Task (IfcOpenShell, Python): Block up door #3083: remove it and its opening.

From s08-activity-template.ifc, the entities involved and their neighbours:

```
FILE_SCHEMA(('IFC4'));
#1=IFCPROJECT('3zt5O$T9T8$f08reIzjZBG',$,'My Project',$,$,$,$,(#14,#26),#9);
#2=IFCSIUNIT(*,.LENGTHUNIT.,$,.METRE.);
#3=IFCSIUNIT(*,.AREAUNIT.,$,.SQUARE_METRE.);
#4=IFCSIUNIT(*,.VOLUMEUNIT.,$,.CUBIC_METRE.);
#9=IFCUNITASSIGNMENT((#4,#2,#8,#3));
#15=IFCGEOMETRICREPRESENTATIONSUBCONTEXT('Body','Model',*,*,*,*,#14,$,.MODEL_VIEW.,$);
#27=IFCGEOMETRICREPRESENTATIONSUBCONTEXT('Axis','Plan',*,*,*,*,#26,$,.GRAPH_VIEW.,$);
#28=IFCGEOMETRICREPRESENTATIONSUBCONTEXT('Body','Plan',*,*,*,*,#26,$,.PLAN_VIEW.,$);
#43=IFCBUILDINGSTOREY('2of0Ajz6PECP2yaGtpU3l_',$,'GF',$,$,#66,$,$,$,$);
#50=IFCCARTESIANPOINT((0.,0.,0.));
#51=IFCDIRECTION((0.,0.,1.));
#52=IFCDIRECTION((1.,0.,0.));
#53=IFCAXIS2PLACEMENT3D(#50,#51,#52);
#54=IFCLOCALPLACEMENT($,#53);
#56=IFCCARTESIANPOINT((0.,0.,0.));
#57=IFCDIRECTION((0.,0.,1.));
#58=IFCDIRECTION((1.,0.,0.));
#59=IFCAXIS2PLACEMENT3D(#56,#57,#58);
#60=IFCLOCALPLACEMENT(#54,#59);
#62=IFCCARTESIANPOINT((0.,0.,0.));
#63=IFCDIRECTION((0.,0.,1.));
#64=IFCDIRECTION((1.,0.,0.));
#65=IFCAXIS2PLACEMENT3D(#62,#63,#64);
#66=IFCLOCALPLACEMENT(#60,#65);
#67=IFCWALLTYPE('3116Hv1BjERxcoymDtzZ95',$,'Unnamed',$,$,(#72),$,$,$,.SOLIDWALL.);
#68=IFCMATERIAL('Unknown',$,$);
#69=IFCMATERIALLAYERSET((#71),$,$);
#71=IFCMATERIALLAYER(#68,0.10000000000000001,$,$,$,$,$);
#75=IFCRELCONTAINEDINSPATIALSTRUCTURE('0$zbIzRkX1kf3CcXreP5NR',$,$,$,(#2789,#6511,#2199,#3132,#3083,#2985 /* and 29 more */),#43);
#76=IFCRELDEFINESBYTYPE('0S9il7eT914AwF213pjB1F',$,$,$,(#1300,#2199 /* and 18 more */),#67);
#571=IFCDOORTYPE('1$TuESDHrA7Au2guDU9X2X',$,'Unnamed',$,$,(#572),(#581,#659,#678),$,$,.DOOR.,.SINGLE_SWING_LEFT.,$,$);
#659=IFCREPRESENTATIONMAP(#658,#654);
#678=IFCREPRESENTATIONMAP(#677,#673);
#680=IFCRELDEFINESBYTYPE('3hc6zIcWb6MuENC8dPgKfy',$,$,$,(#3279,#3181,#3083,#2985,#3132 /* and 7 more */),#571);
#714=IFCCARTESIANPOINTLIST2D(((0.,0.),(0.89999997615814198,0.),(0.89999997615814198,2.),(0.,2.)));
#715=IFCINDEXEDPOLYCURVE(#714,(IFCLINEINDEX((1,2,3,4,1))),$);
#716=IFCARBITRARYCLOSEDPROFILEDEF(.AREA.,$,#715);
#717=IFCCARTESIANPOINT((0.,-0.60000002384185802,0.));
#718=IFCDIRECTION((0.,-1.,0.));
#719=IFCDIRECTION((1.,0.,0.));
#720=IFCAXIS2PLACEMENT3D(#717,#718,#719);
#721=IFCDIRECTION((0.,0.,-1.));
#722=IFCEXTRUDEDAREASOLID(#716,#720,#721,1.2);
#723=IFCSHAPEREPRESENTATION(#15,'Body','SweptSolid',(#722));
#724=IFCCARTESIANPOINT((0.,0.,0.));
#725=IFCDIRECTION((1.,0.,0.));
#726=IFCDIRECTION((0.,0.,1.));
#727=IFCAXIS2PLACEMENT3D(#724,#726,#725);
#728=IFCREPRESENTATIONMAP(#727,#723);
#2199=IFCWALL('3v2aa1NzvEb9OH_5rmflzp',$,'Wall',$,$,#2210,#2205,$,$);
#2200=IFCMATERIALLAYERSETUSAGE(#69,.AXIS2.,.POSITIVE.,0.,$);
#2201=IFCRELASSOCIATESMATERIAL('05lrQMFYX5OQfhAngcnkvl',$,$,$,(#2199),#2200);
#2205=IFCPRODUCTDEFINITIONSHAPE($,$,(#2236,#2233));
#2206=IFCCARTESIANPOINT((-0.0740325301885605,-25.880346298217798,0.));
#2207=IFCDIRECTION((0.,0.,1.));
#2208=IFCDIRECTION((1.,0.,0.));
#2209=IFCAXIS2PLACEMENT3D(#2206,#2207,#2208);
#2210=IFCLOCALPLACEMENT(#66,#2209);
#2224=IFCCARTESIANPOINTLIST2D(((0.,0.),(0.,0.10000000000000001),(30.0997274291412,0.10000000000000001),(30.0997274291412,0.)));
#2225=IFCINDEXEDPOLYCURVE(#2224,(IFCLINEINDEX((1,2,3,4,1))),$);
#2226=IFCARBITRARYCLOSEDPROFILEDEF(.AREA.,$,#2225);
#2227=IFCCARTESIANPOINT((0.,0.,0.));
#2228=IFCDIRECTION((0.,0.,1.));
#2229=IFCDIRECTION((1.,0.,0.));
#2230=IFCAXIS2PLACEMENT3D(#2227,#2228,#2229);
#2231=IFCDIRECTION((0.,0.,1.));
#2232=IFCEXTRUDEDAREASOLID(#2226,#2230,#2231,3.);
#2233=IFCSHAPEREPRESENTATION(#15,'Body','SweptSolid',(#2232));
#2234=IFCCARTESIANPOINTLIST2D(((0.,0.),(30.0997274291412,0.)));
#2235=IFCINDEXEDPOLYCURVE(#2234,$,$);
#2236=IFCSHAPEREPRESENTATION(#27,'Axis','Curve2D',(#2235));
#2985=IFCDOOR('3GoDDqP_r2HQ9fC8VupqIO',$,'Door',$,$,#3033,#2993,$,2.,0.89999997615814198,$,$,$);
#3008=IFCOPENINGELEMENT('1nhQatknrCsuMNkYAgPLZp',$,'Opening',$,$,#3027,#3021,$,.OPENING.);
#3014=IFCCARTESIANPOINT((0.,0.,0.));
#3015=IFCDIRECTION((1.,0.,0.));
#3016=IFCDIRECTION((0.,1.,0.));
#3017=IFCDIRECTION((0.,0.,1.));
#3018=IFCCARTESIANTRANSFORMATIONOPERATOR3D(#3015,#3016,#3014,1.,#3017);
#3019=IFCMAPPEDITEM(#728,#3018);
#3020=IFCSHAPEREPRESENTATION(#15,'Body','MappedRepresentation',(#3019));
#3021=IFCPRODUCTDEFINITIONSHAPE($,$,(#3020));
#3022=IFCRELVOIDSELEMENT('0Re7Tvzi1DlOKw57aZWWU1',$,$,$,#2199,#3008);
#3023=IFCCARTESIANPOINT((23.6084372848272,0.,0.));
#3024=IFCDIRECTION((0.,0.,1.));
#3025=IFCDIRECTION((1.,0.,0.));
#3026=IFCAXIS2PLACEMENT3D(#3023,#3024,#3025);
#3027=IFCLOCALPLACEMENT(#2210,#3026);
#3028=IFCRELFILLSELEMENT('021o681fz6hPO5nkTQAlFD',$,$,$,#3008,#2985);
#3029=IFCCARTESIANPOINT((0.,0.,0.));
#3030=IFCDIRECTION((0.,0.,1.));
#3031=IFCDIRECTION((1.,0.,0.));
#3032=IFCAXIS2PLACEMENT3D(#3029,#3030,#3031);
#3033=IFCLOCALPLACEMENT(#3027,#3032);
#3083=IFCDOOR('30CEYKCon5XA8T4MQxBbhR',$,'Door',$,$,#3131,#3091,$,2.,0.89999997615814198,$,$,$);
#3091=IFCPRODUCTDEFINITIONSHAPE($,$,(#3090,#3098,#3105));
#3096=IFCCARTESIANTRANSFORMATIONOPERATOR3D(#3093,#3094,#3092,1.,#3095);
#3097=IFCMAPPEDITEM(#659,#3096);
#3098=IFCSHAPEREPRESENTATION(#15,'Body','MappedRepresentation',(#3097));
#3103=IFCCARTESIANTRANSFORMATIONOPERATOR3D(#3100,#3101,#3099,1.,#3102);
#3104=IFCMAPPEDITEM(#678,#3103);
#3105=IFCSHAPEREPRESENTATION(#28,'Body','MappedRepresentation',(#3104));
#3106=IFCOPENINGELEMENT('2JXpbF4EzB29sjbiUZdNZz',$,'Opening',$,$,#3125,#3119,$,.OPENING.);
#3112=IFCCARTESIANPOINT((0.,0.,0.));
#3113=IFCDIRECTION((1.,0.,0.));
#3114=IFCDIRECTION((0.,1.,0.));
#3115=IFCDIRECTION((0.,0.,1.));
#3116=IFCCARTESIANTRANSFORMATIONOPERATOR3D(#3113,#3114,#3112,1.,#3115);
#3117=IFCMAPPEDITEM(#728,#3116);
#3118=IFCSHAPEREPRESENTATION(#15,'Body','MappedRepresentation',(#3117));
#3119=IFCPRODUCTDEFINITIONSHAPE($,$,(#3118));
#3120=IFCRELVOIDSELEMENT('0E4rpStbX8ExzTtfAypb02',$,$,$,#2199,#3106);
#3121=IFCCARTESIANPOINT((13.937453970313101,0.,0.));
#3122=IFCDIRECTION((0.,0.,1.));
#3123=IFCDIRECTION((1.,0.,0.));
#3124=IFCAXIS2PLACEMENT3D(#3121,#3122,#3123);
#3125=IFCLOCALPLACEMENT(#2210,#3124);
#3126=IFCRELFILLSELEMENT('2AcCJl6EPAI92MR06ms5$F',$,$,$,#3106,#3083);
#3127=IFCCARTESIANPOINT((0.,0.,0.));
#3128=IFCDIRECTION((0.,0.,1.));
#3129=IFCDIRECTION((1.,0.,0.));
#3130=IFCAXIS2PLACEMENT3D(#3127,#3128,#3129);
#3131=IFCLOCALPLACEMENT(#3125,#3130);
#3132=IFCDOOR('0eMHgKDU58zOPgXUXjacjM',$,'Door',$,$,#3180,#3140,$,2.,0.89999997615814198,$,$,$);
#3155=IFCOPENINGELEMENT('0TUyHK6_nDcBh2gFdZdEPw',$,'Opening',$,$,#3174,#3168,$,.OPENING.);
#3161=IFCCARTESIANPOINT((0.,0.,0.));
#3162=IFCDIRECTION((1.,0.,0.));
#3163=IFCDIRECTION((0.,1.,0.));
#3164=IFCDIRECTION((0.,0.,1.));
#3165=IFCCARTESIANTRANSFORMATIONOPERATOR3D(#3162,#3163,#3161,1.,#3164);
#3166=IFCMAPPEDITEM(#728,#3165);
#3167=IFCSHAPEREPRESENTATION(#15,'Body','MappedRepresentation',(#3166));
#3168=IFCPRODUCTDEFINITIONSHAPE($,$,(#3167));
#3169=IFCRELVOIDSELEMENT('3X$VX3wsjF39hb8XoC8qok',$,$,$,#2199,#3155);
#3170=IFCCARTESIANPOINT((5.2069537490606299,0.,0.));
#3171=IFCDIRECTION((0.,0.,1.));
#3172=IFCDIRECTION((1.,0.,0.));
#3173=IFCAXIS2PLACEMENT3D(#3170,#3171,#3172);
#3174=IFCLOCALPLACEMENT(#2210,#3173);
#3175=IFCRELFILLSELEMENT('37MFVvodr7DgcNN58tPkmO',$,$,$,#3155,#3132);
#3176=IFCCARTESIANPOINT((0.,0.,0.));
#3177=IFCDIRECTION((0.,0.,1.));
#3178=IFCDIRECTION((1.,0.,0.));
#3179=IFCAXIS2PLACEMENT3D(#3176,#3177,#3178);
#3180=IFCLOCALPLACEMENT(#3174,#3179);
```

```python
import ifcopenshell
import ifcopenshell.api.feature
import ifcopenshell.api.root
import ifcopenshell.geom
import ifcopenshell.util.shape

model = ifcopenshell.open("s08-activity-template.ifc")
settings = ifcopenshell.geom.settings()


def volume(element):
    """Net volume in cubic metres, openings subtracted."""
    shape = ifcopenshell.geom.create_shape(settings, element)
    return ifcopenshell.util.shape.get_volume(shape.geometry)


door = model.by_guid("30CEYKCon5XA8T4MQxBbhR")
opening = door.FillsVoids[0].RelatingOpeningElement
wall = opening.VoidsElements[0].RelatingBuildingElement
before = volume(wall)

ifcopenshell.api.root.remove_product(model, product=door)
ifcopenshell.api.feature.remove_feature(model, feature=opening)

after = volume(wall)

print(f"wall volume {before:.3f} -> {after:.3f} m3")

model.write("s08-activity-template_updated.ifc")
```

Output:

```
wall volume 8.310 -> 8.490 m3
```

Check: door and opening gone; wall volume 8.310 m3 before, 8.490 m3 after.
